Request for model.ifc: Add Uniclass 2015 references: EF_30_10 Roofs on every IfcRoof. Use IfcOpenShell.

First a look at what the model holds.

```python
import ifcopenshell

model = ifcopenshell.open("model.ifc")
print(model.schema)
print("classifications:", [c.Name for c in model.by_type("IfcClassification")])
for ifc_class in ("IfcDoor", "IfcRoof", "IfcStair", "IfcWall", "IfcWindow"):
    print(ifc_class, len(model.by_type(ifc_class)))
```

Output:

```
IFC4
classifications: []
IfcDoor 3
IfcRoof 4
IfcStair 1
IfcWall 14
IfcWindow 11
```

```python
import ifcopenshell
import ifcopenshell.api.classification

model = ifcopenshell.open("model.ifc")

system = ifcopenshell.api.classification.add_classification(model, classification="Uniclass 2015")

codes = {
    "IfcRoof": ("EF_30_10", "Roofs"),
}
for ifc_class, (code, name) in codes.items():
    products = model.by_type(ifc_class)
    ifcopenshell.api.classification.add_reference(
        model, products=products, classification=system, identification=code, name=name
    )
    print(code, len(products))

model.write("model_updated.ifc")
```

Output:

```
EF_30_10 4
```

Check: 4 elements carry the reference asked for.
